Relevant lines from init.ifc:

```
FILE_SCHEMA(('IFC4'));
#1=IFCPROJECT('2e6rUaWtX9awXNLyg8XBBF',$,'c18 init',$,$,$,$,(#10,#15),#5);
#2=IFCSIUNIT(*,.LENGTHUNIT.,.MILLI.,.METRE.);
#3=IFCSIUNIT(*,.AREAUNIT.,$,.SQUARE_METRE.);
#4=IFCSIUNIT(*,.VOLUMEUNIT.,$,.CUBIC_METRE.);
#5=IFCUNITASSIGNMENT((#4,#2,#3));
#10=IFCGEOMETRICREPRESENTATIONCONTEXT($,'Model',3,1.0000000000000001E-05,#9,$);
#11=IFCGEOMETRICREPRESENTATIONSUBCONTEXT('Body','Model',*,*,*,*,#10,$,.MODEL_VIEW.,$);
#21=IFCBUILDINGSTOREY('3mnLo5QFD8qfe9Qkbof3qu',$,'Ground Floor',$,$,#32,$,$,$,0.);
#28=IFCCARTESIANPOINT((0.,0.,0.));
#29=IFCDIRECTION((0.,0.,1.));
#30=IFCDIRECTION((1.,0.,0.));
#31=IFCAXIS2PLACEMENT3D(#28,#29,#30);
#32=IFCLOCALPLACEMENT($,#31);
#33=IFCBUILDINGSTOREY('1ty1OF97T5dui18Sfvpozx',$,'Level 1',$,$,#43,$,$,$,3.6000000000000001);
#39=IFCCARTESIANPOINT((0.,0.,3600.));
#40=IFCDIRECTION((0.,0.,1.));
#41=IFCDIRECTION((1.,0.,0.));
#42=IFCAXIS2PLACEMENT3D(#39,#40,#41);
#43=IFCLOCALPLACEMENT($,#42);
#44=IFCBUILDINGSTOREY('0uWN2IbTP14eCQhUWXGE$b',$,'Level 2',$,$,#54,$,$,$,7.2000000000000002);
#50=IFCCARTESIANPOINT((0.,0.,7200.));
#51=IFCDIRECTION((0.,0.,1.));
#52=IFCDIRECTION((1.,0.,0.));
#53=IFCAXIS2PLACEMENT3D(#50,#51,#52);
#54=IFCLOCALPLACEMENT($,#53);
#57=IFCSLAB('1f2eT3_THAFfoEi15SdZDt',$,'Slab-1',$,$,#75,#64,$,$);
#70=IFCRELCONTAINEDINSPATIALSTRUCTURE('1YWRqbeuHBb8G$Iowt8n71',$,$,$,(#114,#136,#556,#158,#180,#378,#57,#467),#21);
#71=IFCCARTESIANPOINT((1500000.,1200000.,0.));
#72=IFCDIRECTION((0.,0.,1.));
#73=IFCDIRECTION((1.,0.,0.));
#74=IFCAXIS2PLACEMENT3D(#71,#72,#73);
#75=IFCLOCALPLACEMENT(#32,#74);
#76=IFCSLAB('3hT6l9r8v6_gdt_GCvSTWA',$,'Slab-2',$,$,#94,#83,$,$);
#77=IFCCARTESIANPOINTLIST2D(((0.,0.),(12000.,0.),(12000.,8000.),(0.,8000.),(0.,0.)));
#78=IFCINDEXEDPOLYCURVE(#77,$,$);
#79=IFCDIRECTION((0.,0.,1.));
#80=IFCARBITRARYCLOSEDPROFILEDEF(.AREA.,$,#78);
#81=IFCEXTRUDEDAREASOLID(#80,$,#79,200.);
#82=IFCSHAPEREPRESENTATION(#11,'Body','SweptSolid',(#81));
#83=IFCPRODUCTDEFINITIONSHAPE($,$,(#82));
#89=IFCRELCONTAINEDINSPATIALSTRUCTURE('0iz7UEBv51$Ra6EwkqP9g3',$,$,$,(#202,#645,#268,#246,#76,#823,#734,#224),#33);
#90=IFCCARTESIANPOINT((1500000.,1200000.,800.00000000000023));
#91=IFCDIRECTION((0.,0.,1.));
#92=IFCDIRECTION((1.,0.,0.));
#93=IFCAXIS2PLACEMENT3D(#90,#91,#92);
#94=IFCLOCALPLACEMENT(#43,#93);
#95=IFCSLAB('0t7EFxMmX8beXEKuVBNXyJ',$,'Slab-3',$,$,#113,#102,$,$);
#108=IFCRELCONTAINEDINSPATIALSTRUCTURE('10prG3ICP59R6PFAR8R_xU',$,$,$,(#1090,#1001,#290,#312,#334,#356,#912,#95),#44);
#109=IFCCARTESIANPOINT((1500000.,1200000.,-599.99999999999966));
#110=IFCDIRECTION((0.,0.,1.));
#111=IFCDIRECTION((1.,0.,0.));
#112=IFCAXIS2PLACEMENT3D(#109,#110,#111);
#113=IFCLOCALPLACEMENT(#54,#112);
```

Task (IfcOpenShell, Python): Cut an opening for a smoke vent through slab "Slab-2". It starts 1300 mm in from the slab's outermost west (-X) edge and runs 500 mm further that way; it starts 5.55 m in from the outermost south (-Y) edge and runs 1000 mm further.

```python
import numpy as np
import ifcopenshell
import ifcopenshell.api.feature
import ifcopenshell.api.geometry
import ifcopenshell.api.root
import ifcopenshell.geom
import ifcopenshell.util.placement
import ifcopenshell.util.representation
import ifcopenshell.util.shape
import ifcopenshell.util.unit

model = ifcopenshell.open("init.ifc")
unit_scale = ifcopenshell.util.unit.calculate_unit_scale(model)
settings = ifcopenshell.geom.settings()


def volume(element):
    """Net volume in cubic metres, openings subtracted."""
    shape = ifcopenshell.geom.create_shape(settings, element)
    return ifcopenshell.util.shape.get_volume(shape.geometry)


slab = model.by_id(76)
before = volume(slab)

# Extent in the slab's own axes, in metres. The edges named are its -X and -Y sides.
slab_shape = ifcopenshell.geom.create_shape(settings, slab)
vertices = ifcopenshell.util.shape.get_vertices(slab_shape.geometry)
x_min, y_min, bottom = vertices.min(axis=0)
top = vertices[:, 2].max()

opening = ifcopenshell.api.root.create_entity(model, ifc_class="IfcOpeningElement", name="Smoke vent opening", predefined_type="OPENING")
context = ifcopenshell.util.representation.get_context(model, "Model", "Body", "MODEL_VIEW")
width, depth = 0.5, 1
outline = [(0.0, 0.0), (width, 0.0), (width, depth), (0.0, depth), (0.0, 0.0)]
# Overshoot both faces by 50 mm so the cut is clean.
shape = ifcopenshell.api.geometry.add_slab_representation(
    model, context=context, depth=top - bottom + 0.1, polyline=outline
)
ifcopenshell.api.geometry.assign_representation(model, product=opening, representation=shape)

matrix = ifcopenshell.util.placement.get_local_placement(slab.ObjectPlacement)
matrix[:, 3] = matrix @ np.append(np.array([x_min + 1.3, y_min + 5.55, bottom - 0.05]) / unit_scale, 1.0)
ifcopenshell.api.geometry.edit_object_placement(model, product=opening, matrix=matrix, is_si=False)
ifcopenshell.api.feature.add_feature(model, feature=opening, element=slab)

after = volume(slab)

print(f"slab volume {before:.3f} -> {after:.3f} m3")

model.write("init_updated.ifc")
```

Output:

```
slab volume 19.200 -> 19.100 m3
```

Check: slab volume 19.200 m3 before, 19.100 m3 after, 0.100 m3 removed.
